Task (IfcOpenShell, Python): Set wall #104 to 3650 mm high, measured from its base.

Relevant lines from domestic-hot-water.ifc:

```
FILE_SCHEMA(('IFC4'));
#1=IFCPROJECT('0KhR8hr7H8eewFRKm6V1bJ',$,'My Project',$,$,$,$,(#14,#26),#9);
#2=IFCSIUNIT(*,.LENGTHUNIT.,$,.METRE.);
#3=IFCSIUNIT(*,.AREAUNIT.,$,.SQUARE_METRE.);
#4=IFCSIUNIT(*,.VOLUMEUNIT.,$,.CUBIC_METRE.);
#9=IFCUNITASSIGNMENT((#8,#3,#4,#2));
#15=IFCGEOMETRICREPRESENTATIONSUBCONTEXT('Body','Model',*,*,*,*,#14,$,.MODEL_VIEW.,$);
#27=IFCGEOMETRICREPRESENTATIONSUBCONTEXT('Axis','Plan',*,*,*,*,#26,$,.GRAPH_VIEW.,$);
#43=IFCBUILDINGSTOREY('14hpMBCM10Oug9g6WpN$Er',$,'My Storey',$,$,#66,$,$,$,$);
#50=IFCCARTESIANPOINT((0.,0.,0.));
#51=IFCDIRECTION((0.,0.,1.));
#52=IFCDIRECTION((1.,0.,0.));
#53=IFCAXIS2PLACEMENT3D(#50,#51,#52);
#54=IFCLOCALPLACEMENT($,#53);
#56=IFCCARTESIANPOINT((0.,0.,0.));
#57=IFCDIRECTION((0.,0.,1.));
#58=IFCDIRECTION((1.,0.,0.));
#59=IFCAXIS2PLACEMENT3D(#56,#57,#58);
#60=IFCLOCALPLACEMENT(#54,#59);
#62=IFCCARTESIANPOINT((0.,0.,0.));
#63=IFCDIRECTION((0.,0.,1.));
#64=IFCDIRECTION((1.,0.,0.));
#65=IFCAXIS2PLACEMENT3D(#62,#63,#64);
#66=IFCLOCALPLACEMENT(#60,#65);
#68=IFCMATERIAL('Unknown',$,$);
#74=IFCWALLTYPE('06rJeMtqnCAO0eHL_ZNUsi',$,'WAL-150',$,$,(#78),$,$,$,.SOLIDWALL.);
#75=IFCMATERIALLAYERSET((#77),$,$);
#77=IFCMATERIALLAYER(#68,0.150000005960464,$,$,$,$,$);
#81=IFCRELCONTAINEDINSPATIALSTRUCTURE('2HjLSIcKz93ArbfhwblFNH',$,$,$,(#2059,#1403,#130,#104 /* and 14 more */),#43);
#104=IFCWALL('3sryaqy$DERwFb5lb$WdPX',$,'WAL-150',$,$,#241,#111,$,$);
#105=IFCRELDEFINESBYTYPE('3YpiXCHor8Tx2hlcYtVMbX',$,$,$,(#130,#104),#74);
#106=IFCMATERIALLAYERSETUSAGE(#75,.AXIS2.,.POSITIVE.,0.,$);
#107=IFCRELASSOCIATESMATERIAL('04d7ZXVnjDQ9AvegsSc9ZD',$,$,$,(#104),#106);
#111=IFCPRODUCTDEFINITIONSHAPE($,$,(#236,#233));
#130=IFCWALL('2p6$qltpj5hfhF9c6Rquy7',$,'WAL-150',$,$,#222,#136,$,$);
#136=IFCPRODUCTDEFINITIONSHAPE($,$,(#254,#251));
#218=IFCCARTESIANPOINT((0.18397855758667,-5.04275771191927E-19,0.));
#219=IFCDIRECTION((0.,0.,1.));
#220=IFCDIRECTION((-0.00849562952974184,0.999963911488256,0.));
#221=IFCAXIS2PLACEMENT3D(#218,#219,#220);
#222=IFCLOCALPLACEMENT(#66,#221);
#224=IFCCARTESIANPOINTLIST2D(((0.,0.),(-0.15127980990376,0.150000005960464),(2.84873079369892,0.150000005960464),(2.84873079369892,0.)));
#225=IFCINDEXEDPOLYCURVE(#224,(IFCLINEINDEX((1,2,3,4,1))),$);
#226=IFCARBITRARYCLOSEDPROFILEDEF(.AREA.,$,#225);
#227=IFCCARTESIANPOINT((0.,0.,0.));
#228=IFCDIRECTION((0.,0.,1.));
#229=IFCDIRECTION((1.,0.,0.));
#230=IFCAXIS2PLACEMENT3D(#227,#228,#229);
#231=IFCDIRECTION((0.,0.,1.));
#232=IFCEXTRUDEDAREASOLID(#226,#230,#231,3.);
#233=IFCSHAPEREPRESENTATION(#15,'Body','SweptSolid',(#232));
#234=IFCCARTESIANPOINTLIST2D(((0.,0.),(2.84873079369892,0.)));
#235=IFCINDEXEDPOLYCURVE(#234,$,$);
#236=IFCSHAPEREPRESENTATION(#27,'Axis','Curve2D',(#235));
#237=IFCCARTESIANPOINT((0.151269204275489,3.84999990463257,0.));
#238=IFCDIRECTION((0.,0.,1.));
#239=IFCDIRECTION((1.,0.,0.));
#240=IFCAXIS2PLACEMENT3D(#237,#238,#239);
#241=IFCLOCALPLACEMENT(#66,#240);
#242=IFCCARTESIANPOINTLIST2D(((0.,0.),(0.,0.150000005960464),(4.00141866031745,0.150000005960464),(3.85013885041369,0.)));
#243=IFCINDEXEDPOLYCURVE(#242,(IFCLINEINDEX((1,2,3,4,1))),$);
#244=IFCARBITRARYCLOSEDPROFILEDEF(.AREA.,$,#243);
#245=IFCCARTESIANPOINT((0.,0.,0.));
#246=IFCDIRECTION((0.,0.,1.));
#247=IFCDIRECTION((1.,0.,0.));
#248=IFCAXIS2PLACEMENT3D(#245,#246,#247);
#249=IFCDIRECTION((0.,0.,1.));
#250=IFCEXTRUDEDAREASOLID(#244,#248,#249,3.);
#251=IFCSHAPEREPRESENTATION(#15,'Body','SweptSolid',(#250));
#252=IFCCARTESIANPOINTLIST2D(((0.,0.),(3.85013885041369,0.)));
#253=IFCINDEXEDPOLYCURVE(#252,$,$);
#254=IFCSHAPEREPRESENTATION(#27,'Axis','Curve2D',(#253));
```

```python
import ifcopenshell
import ifcopenshell.geom
import ifcopenshell.util.representation
import ifcopenshell.util.shape

model = ifcopenshell.open("domestic-hot-water.ifc")
settings = ifcopenshell.geom.settings()


def volume(element):
    """Net volume in cubic metres, openings subtracted."""
    shape = ifcopenshell.geom.create_shape(settings, element)
    return ifcopenshell.util.shape.get_volume(shape.geometry)


wall = model.by_id(104)
before = volume(wall)

body = ifcopenshell.util.representation.get_representation(wall, "Model", "Body")
solid = body.Items[0]
old_height = solid.Depth
solid.Depth = 3.65
after = volume(wall)

print(f"height {old_height:g} -> {solid.Depth:g}, volume {before:.3f} -> {after:.3f} m3")

model.write("domestic-hot-water_v2.ifc")
```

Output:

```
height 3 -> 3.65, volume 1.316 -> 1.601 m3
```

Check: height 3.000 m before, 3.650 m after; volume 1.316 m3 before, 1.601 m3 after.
